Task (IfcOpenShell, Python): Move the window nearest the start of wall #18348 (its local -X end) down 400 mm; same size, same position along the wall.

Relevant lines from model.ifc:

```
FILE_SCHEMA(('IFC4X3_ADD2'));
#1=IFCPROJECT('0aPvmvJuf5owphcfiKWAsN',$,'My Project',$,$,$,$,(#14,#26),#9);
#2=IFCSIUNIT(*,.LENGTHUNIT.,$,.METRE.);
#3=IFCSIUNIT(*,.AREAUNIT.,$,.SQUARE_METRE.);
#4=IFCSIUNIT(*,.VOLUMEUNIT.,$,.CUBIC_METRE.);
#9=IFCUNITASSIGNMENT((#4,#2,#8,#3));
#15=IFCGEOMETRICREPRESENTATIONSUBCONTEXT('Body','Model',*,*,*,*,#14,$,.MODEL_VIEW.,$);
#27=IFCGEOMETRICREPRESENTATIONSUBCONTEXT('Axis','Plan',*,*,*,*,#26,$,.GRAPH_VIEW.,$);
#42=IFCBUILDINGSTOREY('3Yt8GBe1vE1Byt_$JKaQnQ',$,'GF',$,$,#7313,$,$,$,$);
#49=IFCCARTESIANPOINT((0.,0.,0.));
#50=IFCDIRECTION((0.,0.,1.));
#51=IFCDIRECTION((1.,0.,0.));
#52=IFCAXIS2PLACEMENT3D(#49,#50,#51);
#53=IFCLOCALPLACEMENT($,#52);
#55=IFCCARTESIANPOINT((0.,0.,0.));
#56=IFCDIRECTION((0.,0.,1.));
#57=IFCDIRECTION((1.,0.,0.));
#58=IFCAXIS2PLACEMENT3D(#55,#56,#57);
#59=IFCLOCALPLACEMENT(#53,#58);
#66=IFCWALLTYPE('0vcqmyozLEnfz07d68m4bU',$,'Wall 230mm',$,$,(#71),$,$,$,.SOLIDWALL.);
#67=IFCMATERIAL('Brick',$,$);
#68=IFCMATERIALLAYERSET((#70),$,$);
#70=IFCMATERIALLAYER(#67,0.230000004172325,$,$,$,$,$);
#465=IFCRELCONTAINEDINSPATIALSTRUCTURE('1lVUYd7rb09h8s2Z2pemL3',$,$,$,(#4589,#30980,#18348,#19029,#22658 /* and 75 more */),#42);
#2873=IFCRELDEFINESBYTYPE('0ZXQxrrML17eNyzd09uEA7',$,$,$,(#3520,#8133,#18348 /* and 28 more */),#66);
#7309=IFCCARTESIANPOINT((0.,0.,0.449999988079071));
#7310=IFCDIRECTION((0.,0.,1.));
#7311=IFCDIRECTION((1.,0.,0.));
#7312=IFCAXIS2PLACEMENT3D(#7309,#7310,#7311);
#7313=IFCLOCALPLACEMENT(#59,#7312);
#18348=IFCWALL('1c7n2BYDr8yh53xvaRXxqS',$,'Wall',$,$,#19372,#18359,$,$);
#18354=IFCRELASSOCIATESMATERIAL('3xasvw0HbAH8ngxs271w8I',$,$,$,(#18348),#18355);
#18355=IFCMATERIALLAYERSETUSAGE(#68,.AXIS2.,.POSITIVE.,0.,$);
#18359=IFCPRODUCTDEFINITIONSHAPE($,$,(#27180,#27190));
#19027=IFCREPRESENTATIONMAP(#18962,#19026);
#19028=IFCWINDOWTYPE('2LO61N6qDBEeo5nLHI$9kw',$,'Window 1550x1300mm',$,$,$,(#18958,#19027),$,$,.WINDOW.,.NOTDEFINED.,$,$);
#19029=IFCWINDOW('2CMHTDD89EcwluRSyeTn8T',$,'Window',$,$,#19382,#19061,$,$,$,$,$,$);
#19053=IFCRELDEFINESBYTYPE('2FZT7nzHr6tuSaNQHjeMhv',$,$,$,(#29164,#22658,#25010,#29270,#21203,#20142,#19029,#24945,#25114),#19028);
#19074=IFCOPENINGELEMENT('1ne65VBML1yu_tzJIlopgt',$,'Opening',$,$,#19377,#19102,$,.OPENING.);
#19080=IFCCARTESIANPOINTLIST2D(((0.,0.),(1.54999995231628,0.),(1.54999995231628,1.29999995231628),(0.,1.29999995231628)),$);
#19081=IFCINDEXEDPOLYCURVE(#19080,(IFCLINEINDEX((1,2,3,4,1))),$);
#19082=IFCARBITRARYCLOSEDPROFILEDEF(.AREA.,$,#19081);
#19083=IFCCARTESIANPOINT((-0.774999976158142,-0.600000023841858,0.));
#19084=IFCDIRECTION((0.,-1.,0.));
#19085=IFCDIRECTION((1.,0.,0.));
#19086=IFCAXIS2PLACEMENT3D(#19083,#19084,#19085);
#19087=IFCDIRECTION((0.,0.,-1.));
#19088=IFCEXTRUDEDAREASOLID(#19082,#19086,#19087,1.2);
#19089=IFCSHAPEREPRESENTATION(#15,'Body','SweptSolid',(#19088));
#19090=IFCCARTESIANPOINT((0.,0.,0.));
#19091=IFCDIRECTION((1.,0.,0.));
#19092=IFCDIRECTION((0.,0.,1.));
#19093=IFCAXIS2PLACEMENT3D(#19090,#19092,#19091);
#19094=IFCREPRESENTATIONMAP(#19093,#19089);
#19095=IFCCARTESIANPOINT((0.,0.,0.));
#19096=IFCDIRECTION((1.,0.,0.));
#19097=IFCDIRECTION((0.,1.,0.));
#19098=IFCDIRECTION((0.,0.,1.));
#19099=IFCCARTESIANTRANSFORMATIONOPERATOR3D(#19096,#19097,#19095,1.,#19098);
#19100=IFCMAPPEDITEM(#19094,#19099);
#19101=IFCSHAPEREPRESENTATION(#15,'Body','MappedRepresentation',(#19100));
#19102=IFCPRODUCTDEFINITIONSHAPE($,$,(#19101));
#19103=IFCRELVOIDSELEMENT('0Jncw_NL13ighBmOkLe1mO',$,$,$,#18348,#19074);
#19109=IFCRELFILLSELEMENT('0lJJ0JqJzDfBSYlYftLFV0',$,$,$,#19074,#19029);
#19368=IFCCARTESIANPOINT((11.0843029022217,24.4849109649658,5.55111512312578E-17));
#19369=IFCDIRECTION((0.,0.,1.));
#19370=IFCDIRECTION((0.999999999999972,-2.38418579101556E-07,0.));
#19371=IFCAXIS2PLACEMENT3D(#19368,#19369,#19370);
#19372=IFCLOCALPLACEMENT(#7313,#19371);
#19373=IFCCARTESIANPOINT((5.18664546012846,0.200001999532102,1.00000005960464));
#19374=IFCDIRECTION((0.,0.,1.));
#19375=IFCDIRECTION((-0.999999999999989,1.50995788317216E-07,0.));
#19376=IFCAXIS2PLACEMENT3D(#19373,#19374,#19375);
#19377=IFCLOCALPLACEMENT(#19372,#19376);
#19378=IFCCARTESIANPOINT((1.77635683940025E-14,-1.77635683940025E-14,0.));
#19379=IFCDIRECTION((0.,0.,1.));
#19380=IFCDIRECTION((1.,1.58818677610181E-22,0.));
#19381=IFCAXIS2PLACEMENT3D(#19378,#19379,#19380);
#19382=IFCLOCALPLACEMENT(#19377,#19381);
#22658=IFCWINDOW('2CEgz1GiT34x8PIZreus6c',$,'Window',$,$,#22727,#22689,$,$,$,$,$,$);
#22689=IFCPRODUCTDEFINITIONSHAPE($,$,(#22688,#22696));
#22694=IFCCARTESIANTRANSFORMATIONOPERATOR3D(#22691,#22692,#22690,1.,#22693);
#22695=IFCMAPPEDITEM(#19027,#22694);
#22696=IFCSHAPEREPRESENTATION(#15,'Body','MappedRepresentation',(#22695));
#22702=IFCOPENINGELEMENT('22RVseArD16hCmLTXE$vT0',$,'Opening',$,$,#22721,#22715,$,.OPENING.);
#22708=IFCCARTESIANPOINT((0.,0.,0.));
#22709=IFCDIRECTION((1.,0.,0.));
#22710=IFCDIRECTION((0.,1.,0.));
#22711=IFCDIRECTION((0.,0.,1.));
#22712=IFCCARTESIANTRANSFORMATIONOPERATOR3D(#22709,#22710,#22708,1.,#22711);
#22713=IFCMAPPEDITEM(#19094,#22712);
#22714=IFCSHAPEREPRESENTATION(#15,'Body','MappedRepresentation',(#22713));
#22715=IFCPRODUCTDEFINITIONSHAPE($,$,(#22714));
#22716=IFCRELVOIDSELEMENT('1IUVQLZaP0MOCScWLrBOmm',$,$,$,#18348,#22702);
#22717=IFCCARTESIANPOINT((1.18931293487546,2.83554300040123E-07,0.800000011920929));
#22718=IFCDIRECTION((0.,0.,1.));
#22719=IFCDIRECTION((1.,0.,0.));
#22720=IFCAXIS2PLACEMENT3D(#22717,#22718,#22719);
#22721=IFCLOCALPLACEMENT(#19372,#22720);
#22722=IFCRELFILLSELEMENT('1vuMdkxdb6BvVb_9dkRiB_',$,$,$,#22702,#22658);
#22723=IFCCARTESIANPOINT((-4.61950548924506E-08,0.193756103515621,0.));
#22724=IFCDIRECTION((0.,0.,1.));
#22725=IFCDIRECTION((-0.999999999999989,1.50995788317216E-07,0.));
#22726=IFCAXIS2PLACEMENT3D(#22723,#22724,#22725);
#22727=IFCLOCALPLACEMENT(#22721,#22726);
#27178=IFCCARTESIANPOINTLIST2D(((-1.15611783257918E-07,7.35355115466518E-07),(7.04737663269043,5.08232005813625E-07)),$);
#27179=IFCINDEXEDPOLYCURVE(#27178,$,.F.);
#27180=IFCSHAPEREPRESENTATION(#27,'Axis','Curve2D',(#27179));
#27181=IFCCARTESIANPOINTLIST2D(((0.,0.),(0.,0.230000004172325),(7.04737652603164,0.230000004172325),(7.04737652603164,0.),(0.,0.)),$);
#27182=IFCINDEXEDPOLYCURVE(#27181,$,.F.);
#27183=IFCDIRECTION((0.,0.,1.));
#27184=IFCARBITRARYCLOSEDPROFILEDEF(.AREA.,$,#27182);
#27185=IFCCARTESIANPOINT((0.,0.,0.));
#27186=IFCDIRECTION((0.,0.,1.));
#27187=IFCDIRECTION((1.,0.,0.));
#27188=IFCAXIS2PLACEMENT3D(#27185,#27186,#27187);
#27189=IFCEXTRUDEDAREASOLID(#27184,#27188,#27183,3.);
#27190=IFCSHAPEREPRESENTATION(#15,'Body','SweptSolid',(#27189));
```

```python
import numpy as np
import ifcopenshell
import ifcopenshell.api.geometry
import ifcopenshell.util.placement
import ifcopenshell.util.unit

model = ifcopenshell.open("model.ifc")
unit_scale = ifcopenshell.util.unit.calculate_unit_scale(model)

window = model.by_guid("2CEgz1GiT34x8PIZreus6c")
opening = window.FillsVoids[0].RelatingOpeningElement
dz = -0.4 / unit_scale

shift = np.array([0.0, 0.0, dz])
# The window is placed relative to its opening, so it follows when the opening moves.
matrix = ifcopenshell.util.placement.get_local_placement(opening.ObjectPlacement)
matrix[:3, 3] += shift
ifcopenshell.api.geometry.edit_object_placement(
    model, product=opening, matrix=matrix, is_si=False, should_transform_children=True
)

print(f"moved by {dz * unit_scale:+.3f} m")

model.write("model_edited.ifc")
```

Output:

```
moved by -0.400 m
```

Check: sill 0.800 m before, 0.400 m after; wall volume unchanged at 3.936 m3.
